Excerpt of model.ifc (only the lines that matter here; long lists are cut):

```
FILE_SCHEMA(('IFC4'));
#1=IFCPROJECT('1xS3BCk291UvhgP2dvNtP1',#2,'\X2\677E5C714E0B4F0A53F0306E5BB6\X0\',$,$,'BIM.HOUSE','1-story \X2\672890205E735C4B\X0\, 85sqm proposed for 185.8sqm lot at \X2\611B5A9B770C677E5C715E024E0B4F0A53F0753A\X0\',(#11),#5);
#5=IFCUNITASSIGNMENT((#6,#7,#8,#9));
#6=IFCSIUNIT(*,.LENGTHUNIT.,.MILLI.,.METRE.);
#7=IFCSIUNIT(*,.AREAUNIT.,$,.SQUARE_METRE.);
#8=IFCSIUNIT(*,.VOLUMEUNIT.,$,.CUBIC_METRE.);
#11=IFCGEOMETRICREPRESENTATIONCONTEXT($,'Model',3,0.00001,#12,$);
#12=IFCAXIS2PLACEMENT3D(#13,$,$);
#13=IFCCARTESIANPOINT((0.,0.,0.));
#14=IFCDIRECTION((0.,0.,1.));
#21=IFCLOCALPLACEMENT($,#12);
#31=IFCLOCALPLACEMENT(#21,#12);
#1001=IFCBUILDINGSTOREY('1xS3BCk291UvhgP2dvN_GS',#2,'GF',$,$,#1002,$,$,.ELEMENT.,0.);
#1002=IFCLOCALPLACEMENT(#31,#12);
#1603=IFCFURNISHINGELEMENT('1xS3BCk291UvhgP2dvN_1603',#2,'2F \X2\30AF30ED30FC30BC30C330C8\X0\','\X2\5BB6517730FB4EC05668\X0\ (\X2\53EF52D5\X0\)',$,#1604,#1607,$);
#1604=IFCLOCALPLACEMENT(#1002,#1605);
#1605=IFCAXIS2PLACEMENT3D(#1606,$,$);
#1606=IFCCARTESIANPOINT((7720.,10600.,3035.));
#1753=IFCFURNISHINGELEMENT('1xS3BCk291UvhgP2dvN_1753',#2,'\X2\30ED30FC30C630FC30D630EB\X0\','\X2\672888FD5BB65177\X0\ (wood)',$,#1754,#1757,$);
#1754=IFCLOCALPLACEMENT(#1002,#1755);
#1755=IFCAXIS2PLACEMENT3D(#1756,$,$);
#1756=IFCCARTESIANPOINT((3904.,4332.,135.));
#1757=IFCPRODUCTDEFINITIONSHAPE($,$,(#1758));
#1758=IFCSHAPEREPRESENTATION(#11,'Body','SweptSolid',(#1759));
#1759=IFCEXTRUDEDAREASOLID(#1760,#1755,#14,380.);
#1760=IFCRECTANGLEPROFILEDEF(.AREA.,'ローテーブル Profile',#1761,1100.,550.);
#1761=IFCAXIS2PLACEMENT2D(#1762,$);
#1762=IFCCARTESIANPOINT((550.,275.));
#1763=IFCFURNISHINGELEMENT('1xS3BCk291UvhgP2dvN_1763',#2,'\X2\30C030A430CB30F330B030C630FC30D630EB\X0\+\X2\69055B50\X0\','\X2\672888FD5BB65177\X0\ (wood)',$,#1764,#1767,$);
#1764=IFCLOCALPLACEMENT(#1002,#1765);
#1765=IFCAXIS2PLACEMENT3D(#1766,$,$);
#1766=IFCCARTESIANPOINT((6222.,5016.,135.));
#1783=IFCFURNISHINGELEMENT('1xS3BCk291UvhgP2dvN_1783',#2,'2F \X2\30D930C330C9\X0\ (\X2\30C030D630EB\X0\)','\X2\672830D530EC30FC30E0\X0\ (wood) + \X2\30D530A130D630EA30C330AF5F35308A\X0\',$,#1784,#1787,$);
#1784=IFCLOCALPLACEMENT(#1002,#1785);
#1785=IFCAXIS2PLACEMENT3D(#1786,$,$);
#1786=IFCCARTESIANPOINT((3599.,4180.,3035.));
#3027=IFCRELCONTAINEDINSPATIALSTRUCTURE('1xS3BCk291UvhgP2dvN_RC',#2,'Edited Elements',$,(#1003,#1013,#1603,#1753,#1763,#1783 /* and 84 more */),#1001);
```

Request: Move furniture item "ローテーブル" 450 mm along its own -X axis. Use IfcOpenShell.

```python
import ifcopenshell
import ifcopenshell.api.geometry
import ifcopenshell.util.placement
import ifcopenshell.util.unit

model = ifcopenshell.open("model.ifc")
unit_scale = ifcopenshell.util.unit.calculate_unit_scale(model)

item = model.by_guid("1xS3BCk291UvhgP2dvN_1753")
matrix = ifcopenshell.util.placement.get_local_placement(item.ObjectPlacement)
matrix[:3, 3] -= matrix[:3, 0] * 0.45 / unit_scale
ifcopenshell.api.geometry.edit_object_placement(model, product=item, matrix=matrix, is_si=False)

print(ifcopenshell.util.placement.get_local_placement(item.ObjectPlacement).round(3) + 0.0)

model.write("model_edited.ifc")
```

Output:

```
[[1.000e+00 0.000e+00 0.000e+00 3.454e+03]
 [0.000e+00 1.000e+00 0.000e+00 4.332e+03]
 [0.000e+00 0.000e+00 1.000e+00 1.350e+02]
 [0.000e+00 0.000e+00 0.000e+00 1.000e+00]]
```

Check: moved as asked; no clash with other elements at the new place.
